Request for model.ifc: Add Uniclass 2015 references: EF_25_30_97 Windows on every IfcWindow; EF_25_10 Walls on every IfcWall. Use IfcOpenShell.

First a look at what the model holds.

```python
import ifcopenshell

model = ifcopenshell.open("model.ifc")
print(model.schema)
print("classifications:", [c.Name for c in model.by_type("IfcClassification")])
for ifc_class in ("IfcDoor", "IfcRoof", "IfcStair", "IfcWall", "IfcWindow"):
    print(ifc_class, len(model.by_type(ifc_class)))
```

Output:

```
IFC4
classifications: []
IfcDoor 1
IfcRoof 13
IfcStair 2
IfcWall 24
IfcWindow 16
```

```python
import ifcopenshell
import ifcopenshell.api.classification

model = ifcopenshell.open("model.ifc")

system = ifcopenshell.api.classification.add_classification(model, classification="Uniclass 2015")

codes = {
    "IfcWindow": ("EF_25_30_97", "Windows"),
    "IfcWall": ("EF_25_10", "Walls"),
}
for ifc_class, (code, name) in codes.items():
    products = model.by_type(ifc_class)
    ifcopenshell.api.classification.add_reference(
        model, products=products, classification=system, identification=code, name=name
    )
    print(code, len(products))

model.write("model_v2.ifc")
```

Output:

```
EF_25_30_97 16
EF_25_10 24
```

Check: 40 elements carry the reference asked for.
